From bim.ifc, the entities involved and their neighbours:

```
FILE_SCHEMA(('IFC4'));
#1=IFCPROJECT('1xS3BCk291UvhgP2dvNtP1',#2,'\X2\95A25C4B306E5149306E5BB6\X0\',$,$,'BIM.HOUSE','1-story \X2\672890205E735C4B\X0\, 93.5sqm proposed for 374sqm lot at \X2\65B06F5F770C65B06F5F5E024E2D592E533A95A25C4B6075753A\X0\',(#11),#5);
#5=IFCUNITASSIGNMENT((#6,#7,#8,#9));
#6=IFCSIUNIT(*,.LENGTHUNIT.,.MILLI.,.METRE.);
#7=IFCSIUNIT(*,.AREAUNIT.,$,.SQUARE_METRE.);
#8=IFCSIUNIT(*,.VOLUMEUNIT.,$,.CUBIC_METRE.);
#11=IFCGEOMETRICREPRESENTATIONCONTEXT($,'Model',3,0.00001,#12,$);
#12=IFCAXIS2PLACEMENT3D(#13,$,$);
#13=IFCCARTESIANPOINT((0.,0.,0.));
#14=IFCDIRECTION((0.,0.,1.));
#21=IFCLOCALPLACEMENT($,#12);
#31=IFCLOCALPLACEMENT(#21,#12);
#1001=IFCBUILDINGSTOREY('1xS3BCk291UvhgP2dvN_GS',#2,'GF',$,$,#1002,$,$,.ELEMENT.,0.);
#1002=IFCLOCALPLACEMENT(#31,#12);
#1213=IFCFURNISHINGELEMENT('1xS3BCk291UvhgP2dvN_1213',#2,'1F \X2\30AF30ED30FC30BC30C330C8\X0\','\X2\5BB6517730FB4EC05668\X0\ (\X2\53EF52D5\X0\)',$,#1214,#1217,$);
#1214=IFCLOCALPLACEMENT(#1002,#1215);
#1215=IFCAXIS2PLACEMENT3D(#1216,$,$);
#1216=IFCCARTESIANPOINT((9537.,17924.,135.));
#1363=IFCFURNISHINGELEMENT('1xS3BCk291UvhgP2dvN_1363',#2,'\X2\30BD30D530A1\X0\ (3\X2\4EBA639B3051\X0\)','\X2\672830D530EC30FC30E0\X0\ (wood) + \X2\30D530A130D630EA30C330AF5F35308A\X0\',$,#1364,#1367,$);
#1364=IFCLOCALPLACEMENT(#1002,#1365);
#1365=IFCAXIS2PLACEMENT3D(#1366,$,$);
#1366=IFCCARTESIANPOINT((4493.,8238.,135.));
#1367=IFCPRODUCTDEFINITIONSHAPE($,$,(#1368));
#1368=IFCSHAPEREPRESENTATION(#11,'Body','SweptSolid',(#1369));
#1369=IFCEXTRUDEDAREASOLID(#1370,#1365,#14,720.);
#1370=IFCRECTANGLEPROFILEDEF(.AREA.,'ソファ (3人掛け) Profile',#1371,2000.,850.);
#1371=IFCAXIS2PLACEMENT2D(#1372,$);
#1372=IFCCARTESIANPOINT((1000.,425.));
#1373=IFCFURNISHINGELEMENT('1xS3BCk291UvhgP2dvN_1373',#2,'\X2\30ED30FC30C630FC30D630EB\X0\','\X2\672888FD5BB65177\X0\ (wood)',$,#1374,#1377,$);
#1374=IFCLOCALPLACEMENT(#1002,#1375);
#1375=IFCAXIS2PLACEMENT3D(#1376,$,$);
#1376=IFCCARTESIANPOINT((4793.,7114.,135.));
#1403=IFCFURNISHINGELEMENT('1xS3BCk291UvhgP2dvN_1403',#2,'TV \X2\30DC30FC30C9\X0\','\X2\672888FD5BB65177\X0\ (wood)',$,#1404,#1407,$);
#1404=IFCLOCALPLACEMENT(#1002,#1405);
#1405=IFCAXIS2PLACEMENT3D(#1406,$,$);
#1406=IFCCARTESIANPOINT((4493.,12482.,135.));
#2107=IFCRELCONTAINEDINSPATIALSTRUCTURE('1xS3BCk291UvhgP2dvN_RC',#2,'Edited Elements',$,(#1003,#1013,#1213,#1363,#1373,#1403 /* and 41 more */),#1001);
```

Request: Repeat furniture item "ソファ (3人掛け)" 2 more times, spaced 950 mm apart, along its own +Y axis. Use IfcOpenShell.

```python
import ifcopenshell
import ifcopenshell.api.geometry
import ifcopenshell.api.root
import ifcopenshell.util.element
import ifcopenshell.util.placement
import ifcopenshell.util.unit

model = ifcopenshell.open("bim.ifc")
unit_scale = ifcopenshell.util.unit.calculate_unit_scale(model)


def reuse_history(source, copy):
    """copy_class also copies each property set's owner history, people and application; keep the originals."""
    for rel in copy.IsDefinedBy:
        if rel.is_a("IfcRelDefinesByProperties") and (history := rel.RelatingPropertyDefinition.OwnerHistory):
            rel.RelatingPropertyDefinition.OwnerHistory = source.OwnerHistory
            ifcopenshell.util.element.remove_deep2(model, history)


source = model.by_guid("1xS3BCk291UvhgP2dvN_1363")
base = ifcopenshell.util.placement.get_local_placement(source.ObjectPlacement)
step = base[:3, 1] * 0.95 / unit_scale

for i in range(1, 3):
    copy = ifcopenshell.api.root.copy_class(model, product=source)
    copy.Representation = ifcopenshell.util.element.copy_deep(
        model, source.Representation, exclude=["IfcGeometricRepresentationContext", "IfcRepresentationMap"]
    )
    reuse_history(source, copy)
    matrix = base.copy()
    matrix[:3, 3] += i * step
    print("added at", matrix[:3, 3].round(3) + 0.0)
    ifcopenshell.api.geometry.edit_object_placement(model, product=copy, matrix=matrix, is_si=False)

model.write("bim_updated.ifc")
```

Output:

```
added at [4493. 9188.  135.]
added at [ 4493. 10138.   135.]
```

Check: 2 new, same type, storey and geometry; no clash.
